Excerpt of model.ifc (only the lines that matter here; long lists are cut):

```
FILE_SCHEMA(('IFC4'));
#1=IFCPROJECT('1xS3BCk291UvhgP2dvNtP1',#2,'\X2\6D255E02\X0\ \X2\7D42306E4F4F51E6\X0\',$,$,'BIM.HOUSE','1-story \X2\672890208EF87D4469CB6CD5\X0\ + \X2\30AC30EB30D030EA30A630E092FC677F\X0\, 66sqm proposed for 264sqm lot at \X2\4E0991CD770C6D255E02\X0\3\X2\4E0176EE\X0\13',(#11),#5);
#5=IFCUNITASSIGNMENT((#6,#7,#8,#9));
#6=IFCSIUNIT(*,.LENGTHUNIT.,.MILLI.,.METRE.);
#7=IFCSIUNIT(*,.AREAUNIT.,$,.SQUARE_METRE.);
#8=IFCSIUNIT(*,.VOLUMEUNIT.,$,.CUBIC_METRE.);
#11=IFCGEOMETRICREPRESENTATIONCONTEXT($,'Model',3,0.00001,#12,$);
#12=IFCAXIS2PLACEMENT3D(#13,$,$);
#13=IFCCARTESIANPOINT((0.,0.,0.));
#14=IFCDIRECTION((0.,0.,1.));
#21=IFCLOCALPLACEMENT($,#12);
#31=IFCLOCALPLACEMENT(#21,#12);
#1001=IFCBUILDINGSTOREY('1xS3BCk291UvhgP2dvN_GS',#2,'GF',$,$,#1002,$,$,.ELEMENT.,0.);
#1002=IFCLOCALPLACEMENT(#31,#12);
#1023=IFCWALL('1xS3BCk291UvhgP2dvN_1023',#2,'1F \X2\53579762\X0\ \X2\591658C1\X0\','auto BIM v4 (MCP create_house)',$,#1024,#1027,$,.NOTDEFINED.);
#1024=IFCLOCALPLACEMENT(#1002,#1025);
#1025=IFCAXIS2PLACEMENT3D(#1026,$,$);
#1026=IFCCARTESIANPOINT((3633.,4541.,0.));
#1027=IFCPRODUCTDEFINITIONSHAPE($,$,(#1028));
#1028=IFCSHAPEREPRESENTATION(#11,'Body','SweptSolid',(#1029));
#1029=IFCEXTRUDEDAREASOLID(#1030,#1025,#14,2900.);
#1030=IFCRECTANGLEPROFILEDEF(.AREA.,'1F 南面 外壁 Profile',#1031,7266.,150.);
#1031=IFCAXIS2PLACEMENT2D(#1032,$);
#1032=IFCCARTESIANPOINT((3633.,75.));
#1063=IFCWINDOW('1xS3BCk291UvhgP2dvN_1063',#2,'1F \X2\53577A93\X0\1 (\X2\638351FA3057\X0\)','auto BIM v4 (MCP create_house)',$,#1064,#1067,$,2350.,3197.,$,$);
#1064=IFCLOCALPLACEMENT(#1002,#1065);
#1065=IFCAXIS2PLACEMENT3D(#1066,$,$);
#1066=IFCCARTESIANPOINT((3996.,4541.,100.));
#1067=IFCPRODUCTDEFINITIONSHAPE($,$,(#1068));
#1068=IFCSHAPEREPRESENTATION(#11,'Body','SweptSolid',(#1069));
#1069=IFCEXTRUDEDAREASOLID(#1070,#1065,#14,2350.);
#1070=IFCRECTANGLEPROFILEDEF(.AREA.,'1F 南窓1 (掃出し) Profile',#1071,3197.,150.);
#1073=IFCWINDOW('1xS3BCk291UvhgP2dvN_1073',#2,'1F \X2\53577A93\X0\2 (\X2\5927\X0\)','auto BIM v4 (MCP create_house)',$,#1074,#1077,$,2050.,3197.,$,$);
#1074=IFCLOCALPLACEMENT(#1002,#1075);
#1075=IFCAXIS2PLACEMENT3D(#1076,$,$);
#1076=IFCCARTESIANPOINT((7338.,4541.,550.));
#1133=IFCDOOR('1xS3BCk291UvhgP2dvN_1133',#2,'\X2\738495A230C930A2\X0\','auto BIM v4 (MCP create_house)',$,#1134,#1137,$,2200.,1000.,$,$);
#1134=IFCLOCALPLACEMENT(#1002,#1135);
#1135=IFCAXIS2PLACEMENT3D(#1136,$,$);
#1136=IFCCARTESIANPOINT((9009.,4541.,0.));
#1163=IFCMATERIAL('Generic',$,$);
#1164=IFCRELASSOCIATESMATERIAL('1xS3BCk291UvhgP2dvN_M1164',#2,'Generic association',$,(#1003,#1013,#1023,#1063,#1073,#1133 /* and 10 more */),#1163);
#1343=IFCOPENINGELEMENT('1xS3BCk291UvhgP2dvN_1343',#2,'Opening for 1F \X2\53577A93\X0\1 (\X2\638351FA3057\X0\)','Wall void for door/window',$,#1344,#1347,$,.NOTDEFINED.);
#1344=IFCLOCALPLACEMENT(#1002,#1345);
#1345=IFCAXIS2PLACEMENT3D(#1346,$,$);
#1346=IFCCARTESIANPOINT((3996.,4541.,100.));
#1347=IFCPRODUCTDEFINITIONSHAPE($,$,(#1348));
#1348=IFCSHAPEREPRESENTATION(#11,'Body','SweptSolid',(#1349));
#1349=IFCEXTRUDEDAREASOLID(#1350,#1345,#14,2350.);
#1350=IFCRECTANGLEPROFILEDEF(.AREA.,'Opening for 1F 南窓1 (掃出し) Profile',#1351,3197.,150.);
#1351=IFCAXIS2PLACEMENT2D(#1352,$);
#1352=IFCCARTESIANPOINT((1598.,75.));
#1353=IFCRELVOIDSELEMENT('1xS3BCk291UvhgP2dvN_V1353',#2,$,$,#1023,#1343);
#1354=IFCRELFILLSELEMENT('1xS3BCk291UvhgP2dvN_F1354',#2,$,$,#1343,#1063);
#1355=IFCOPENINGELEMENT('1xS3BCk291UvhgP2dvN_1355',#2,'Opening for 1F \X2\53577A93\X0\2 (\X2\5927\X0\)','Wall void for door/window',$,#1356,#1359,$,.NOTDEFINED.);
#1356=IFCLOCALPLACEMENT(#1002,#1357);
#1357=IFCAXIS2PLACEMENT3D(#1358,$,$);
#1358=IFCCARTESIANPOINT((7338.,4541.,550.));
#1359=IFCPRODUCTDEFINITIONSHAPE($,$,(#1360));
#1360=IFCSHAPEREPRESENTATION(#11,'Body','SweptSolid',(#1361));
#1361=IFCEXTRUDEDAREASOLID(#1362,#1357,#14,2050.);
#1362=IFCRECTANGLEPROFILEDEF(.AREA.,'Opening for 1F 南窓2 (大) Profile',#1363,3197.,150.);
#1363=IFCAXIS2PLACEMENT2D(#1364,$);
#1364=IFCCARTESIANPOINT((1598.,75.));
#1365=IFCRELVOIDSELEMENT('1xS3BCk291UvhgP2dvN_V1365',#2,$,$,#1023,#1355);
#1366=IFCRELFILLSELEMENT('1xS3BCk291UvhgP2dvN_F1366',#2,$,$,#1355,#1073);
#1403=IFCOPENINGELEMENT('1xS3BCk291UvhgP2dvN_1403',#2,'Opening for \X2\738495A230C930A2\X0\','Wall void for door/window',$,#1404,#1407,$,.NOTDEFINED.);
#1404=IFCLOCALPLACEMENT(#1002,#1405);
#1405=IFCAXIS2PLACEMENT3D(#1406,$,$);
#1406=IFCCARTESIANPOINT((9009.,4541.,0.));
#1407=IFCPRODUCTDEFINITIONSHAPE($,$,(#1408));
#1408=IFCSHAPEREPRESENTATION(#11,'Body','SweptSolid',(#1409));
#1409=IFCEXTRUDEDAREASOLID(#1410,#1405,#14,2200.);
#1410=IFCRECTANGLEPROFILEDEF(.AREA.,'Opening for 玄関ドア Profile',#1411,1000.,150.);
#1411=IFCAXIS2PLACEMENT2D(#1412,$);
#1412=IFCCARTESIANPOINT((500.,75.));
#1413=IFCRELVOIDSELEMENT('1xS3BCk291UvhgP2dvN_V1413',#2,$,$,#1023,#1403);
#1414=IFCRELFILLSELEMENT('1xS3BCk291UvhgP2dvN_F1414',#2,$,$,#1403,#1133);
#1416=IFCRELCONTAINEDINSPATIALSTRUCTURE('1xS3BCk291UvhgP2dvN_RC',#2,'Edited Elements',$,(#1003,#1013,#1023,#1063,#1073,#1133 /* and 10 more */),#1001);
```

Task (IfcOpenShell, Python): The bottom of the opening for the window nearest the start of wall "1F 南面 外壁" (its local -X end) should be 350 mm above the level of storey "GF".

```python
import numpy as np
import ifcopenshell
import ifcopenshell.api.geometry
import ifcopenshell.geom
import ifcopenshell.util.element
import ifcopenshell.util.placement
import ifcopenshell.util.shape
import ifcopenshell.util.unit

model = ifcopenshell.open("model.ifc")
unit_scale = ifcopenshell.util.unit.calculate_unit_scale(model)

window = model.by_id(1063)
opening = window.FillsVoids[0].RelatingOpeningElement
storey = ifcopenshell.util.element.get_container(window, ifc_class="IfcBuildingStorey")
level = ifcopenshell.util.placement.get_local_placement(storey.ObjectPlacement)[2, 3]

# The opening's origin need not be at the sill, so measure its lowest point.
shape = ifcopenshell.geom.create_shape(ifcopenshell.geom.settings(), opening)
bottom = ifcopenshell.util.shape.get_shape_bottom_elevation(shape, shape.geometry) / unit_scale
dz = level + 0.35 / unit_scale - bottom

shift = np.array([0.0, 0.0, dz])
# The window is not placed relative to its opening, so move both.
for product in (opening, window):
    matrix = ifcopenshell.util.placement.get_local_placement(product.ObjectPlacement)
    matrix[:3, 3] += shift
    ifcopenshell.api.geometry.edit_object_placement(model, product=product, matrix=matrix, is_si=False)

print(f"moved by {dz * unit_scale:+.3f} m")

model.write("model_rev.ifc")
```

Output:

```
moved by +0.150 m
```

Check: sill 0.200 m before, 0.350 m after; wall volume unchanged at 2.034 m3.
